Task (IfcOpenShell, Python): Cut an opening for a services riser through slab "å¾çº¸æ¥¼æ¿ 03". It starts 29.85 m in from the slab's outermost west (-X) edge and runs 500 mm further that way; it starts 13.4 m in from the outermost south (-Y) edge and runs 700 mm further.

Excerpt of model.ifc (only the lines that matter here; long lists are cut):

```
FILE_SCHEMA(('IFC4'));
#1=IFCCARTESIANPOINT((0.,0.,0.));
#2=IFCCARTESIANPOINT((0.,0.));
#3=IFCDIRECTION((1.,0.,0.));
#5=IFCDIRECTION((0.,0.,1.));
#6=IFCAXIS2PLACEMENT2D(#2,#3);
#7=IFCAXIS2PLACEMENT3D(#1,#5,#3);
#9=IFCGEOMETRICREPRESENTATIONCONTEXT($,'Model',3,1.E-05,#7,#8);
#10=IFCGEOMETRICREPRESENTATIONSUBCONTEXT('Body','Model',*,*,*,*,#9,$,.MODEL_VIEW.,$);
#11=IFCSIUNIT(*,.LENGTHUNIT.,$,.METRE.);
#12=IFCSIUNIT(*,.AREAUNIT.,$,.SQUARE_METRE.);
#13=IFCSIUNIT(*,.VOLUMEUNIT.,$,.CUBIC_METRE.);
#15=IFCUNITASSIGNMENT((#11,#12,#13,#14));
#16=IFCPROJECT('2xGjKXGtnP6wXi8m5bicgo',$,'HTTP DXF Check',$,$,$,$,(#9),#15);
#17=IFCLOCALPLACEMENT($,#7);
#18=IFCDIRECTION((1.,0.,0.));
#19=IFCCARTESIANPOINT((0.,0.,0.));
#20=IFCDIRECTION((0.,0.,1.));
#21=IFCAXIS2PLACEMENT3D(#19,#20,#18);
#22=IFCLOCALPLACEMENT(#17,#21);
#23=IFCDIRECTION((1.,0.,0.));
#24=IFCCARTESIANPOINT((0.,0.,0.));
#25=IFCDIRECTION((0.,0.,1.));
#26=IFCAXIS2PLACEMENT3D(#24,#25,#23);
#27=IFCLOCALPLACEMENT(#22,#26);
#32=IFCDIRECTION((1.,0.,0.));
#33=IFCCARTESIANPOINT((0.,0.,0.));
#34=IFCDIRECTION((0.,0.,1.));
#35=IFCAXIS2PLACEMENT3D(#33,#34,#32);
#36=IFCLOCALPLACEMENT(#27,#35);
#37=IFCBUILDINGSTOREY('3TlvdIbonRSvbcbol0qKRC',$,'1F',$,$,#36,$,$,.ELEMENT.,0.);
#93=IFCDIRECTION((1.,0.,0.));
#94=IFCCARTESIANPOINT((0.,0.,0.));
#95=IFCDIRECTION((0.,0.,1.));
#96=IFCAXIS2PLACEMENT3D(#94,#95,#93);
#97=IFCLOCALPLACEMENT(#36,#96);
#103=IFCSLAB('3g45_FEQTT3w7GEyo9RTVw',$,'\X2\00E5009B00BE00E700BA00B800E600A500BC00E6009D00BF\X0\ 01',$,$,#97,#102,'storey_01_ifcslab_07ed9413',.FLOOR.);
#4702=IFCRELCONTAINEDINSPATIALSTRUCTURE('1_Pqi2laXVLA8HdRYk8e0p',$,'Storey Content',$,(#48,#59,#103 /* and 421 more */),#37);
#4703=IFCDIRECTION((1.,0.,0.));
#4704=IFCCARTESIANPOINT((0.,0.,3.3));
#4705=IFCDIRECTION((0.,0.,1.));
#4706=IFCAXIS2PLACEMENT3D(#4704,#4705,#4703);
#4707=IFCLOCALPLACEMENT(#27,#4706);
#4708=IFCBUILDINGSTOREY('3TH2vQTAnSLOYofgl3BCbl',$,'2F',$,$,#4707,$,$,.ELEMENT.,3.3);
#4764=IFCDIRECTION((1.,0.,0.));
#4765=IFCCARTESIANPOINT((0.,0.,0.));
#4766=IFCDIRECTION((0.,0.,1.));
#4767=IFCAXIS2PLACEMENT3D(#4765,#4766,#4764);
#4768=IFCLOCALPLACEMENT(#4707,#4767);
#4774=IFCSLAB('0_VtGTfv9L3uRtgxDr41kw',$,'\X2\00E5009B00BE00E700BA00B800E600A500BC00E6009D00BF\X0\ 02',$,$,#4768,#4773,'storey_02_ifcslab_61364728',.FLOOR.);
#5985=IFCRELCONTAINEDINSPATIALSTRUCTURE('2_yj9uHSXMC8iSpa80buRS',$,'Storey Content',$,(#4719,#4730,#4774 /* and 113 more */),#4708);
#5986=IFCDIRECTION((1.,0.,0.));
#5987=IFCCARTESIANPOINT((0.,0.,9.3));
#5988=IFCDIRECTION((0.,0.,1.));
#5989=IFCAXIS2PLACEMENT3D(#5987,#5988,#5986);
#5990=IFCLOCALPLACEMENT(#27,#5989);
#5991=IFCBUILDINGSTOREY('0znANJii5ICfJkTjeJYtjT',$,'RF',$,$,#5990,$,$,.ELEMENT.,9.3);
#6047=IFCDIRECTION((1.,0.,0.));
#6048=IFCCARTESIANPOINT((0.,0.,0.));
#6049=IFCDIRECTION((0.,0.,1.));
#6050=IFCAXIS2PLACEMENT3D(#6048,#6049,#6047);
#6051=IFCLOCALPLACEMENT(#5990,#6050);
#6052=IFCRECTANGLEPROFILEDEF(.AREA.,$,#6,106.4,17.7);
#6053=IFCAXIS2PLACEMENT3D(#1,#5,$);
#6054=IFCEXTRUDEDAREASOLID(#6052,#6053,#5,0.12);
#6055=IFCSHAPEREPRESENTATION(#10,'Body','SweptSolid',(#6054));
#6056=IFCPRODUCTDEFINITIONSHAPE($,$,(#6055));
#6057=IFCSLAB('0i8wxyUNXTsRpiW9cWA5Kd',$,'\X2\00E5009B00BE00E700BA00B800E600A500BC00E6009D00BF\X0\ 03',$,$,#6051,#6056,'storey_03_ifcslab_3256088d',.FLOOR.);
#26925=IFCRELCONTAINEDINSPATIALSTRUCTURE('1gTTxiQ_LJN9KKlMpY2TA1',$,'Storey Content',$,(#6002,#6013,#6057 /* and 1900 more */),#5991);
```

```python
import numpy as np
import ifcopenshell
import ifcopenshell.api.feature
import ifcopenshell.api.geometry
import ifcopenshell.api.root
import ifcopenshell.geom
import ifcopenshell.util.placement
import ifcopenshell.util.representation
import ifcopenshell.util.shape
import ifcopenshell.util.unit

model = ifcopenshell.open("model.ifc")
unit_scale = ifcopenshell.util.unit.calculate_unit_scale(model)
settings = ifcopenshell.geom.settings()


def volume(element):
    """Net volume in cubic metres, openings subtracted."""
    shape = ifcopenshell.geom.create_shape(settings, element)
    return ifcopenshell.util.shape.get_volume(shape.geometry)


slab = model.by_guid("0i8wxyUNXTsRpiW9cWA5Kd")
before = volume(slab)

# Extent in the slab's own axes, in metres. The edges named are its -X and -Y sides.
slab_shape = ifcopenshell.geom.create_shape(settings, slab)
vertices = ifcopenshell.util.shape.get_vertices(slab_shape.geometry)
x_min, y_min, bottom = vertices.min(axis=0)
top = vertices[:, 2].max()

opening = ifcopenshell.api.root.create_entity(model, ifc_class="IfcOpeningElement", name="Services riser opening", predefined_type="OPENING")
context = ifcopenshell.util.representation.get_context(model, "Model", "Body", "MODEL_VIEW")
width, depth = 0.5, 0.7
outline = [(0.0, 0.0), (width, 0.0), (width, depth), (0.0, depth), (0.0, 0.0)]
# Overshoot both faces by 50 mm so the cut is clean.
shape = ifcopenshell.api.geometry.add_slab_representation(
    model, context=context, depth=top - bottom + 0.1, polyline=outline
)
ifcopenshell.api.geometry.assign_representation(model, product=opening, representation=shape)

matrix = ifcopenshell.util.placement.get_local_placement(slab.ObjectPlacement)
matrix[:, 3] = matrix @ np.append(np.array([x_min + 29.85, y_min + 13.4, bottom - 0.05]) / unit_scale, 1.0)
ifcopenshell.api.geometry.edit_object_placement(model, product=opening, matrix=matrix, is_si=False)
ifcopenshell.api.feature.add_feature(model, feature=opening, element=slab)

after = volume(slab)

print(f"slab volume {before:.3f} -> {after:.3f} m3")

model.write("model_edited.ifc")
```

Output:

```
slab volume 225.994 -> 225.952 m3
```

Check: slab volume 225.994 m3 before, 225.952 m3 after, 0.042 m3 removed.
